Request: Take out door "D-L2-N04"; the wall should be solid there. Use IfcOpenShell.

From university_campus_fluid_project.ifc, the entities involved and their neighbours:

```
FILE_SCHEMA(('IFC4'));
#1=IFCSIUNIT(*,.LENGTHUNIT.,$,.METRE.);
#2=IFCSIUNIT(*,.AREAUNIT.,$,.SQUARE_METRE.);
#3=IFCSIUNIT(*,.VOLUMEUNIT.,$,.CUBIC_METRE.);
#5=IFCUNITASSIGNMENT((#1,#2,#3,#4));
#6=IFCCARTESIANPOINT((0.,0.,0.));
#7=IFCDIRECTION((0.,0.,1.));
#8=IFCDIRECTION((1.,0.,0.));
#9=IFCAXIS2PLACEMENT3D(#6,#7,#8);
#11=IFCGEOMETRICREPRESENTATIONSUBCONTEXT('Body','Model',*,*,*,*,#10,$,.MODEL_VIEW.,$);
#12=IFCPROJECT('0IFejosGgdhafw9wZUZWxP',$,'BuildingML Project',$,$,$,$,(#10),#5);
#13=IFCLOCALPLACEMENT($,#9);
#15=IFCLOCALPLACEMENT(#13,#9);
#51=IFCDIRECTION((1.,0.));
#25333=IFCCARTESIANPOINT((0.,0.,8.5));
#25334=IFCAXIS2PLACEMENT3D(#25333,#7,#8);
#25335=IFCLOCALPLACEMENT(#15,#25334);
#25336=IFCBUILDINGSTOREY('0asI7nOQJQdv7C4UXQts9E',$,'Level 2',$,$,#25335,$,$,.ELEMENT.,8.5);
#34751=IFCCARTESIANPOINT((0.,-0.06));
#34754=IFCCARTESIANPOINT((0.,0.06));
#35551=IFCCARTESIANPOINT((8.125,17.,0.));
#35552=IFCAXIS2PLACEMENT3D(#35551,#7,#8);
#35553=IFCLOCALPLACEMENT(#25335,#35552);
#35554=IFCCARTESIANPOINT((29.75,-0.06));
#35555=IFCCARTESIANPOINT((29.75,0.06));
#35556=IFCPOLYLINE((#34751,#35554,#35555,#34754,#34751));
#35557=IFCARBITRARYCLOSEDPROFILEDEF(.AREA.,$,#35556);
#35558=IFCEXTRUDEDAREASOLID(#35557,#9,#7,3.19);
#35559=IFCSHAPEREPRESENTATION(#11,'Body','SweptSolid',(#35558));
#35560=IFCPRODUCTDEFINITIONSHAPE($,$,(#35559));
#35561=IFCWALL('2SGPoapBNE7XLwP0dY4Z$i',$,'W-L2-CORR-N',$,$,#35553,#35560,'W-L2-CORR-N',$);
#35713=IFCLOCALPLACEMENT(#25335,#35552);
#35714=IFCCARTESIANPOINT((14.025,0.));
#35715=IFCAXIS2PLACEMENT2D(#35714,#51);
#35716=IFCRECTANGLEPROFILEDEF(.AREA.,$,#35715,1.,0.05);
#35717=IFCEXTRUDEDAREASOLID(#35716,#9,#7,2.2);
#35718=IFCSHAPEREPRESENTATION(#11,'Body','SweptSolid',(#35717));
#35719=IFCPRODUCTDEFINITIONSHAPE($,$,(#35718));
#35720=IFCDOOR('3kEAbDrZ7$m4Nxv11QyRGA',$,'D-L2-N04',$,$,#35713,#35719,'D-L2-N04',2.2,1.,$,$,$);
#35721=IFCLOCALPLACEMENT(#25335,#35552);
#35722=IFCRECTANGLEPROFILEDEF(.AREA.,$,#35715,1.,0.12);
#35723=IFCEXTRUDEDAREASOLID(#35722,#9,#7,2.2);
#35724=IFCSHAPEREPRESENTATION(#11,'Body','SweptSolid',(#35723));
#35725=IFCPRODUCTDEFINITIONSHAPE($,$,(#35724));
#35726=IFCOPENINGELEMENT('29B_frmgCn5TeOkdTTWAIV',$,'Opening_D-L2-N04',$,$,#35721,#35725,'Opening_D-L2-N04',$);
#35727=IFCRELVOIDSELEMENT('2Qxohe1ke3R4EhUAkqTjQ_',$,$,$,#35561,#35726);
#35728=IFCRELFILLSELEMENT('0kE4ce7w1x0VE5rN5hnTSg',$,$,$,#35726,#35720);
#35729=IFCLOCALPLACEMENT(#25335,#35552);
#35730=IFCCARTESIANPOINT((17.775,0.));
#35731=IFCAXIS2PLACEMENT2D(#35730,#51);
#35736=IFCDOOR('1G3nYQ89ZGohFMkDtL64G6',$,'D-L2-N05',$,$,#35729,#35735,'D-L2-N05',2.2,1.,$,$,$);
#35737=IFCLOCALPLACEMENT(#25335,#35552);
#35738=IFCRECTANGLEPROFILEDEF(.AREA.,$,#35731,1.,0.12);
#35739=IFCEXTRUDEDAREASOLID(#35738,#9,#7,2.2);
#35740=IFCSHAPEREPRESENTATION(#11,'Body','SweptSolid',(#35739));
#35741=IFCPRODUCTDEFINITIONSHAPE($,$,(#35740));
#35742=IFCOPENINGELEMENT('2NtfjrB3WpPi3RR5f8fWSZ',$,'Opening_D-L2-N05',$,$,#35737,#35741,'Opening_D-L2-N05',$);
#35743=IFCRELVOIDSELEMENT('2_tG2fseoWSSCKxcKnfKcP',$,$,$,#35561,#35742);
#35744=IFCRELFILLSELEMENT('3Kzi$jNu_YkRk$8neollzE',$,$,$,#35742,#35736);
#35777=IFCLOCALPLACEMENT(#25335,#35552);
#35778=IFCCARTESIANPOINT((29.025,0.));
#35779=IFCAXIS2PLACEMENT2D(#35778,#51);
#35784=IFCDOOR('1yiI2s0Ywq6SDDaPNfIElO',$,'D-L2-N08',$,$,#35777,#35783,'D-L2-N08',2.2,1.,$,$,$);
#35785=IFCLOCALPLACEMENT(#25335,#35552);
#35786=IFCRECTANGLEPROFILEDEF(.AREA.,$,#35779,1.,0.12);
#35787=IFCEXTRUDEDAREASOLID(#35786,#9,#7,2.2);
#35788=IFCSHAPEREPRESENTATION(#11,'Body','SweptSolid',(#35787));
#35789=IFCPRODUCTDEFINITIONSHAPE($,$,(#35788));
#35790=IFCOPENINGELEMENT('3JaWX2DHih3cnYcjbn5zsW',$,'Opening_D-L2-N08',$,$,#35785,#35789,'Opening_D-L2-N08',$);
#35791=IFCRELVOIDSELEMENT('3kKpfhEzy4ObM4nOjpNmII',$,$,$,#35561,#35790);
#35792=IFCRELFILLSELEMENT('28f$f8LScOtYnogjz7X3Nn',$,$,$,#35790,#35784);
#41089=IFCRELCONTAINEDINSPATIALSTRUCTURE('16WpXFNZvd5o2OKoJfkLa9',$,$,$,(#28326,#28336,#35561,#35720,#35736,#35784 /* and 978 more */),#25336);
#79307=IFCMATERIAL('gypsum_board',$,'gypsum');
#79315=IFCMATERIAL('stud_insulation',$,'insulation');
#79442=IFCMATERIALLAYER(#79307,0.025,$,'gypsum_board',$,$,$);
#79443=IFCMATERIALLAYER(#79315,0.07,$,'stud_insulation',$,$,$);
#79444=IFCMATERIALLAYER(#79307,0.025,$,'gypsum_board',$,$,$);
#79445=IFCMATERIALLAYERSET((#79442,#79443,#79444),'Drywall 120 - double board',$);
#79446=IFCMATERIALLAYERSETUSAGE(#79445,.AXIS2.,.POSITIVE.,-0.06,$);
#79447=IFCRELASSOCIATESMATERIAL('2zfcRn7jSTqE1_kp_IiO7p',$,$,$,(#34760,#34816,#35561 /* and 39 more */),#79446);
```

```python
import ifcopenshell
import ifcopenshell.api.feature
import ifcopenshell.api.root
import ifcopenshell.geom
import ifcopenshell.util.shape

model = ifcopenshell.open("university_campus_fluid_project.ifc")
settings = ifcopenshell.geom.settings()


def volume(element):
    """Net volume in cubic metres, openings subtracted."""
    shape = ifcopenshell.geom.create_shape(settings, element)
    return ifcopenshell.util.shape.get_volume(shape.geometry)


door = model.by_guid("3kEAbDrZ7$m4Nxv11QyRGA")
opening = door.FillsVoids[0].RelatingOpeningElement
wall = opening.VoidsElements[0].RelatingBuildingElement
before = volume(wall)

ifcopenshell.api.root.remove_product(model, product=door)
ifcopenshell.api.feature.remove_feature(model, feature=opening)

after = volume(wall)

print(f"wall volume {before:.3f} -> {after:.3f} m3")

model.write("university_campus_fluid_project_rev.ifc")
```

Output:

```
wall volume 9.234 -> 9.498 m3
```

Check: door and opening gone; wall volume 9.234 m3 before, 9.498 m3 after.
